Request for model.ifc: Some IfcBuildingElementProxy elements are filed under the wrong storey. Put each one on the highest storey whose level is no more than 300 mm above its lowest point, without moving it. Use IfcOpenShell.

First a look at what the model holds.

```python
import ifcopenshell
import ifcopenshell.util.element
import ifcopenshell.util.placement

model = ifcopenshell.open("model.ifc")
print(model.schema)
for storey in model.by_type("IfcBuildingStorey"):
    level = ifcopenshell.util.placement.get_storey_elevation(storey)
    count = sum(e.is_a("IfcBuildingElementProxy") for e in ifcopenshell.util.element.get_contained(storey))
    print(storey.id(), storey.Name, round(level, 3), count, sep=" | ")
```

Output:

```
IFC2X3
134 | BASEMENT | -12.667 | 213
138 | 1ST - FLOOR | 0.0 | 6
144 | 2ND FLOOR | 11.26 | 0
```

```python
import ifcopenshell
import ifcopenshell.api.spatial
import ifcopenshell.geom
import ifcopenshell.util.element
import ifcopenshell.util.placement
import ifcopenshell.util.shape
import ifcopenshell.util.unit

model = ifcopenshell.open("model.ifc")
unit_scale = ifcopenshell.util.unit.calculate_unit_scale(model)
settings = ifcopenshell.geom.settings()

levels = sorted(
    ((ifcopenshell.util.placement.get_storey_elevation(s) * unit_scale, s) for s in model.by_type("IfcBuildingStorey")),
    key=lambda pair: pair[0],
)

for e in model.by_type("IfcBuildingElementProxy"):
    current = e.ContainedInStructure[0].RelatingStructure if e.ContainedInStructure else None
    if current is None or not current.is_a("IfcBuildingStorey"):
        continue
    shape = ifcopenshell.geom.create_shape(settings, e)
    bottom = ifcopenshell.util.shape.get_shape_bottom_elevation(shape, shape.geometry)
    below = [s for level, s in levels if level <= bottom + 0.3]
    storey = below[-1] if below else levels[0][1]
    if storey != current:
        # assign_container keeps the world position.
        ifcopenshell.api.spatial.assign_container(model, products=[e], relating_structure=storey)
        print(e.id(), current.Name, "->", storey.Name)

model.write("model-out.ifc")
```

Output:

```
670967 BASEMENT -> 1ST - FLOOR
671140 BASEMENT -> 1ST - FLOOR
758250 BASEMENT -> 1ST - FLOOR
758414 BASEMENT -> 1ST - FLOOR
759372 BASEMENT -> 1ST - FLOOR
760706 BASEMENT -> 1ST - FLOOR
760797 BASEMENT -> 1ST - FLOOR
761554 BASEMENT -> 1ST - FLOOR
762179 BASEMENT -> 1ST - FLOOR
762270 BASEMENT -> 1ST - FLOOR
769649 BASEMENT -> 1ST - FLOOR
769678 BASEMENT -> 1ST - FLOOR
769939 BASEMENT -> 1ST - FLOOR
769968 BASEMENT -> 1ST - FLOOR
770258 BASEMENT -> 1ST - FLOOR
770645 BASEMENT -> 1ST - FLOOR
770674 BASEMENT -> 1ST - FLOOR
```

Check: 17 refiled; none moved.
